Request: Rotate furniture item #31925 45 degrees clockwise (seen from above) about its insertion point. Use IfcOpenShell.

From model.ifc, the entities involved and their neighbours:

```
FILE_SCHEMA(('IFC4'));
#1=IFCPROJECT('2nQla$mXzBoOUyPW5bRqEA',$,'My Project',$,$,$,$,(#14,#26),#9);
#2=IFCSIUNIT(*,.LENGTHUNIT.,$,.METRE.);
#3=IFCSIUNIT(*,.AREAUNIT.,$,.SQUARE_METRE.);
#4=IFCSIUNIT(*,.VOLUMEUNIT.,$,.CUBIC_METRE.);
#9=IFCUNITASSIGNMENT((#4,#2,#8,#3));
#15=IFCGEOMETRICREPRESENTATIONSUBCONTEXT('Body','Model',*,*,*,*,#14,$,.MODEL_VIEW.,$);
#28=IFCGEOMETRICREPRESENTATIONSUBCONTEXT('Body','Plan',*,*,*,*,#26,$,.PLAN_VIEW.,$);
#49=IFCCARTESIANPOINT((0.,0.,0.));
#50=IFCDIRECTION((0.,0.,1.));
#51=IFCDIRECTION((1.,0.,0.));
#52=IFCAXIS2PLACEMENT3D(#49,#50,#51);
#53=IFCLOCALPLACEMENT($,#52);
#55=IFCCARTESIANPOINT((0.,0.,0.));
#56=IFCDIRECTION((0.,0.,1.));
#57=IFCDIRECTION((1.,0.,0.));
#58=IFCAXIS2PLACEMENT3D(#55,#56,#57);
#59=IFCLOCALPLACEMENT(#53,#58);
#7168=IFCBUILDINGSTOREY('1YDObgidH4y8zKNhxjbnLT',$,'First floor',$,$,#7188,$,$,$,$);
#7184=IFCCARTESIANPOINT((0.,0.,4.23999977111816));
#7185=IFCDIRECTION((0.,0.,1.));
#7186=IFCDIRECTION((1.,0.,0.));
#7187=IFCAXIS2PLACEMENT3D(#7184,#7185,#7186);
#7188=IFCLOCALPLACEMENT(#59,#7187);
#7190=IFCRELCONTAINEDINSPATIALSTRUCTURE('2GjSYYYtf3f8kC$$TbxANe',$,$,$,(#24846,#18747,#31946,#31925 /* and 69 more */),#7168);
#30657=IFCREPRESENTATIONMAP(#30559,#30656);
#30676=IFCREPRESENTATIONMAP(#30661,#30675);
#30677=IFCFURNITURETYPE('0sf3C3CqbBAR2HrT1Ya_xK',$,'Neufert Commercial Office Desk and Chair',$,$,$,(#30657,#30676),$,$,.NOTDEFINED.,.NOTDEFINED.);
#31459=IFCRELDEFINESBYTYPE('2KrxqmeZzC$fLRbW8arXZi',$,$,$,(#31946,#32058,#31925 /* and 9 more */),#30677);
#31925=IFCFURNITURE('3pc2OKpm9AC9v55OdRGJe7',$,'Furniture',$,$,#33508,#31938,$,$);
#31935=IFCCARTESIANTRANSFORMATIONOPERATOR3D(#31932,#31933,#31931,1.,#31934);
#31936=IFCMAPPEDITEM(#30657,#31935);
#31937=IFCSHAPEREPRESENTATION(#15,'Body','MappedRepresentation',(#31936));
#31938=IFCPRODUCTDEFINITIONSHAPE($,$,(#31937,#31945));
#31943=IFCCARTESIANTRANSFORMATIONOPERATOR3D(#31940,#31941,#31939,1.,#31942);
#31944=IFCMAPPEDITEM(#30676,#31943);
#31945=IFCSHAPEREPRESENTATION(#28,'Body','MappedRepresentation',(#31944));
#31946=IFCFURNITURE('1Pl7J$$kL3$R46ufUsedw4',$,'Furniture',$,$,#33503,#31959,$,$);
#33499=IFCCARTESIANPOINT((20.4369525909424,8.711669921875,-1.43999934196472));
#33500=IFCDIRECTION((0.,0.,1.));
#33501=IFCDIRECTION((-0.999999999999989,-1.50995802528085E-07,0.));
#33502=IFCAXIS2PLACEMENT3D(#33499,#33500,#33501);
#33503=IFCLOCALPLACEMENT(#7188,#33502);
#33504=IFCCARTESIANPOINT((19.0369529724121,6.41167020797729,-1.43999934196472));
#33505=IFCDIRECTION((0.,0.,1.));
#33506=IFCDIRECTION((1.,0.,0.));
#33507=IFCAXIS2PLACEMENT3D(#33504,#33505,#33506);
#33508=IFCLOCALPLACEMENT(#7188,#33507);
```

```python
import ifcopenshell
import ifcopenshell.api.geometry
import ifcopenshell.util.placement

model = ifcopenshell.open("model.ifc")

item = model.by_guid("3pc2OKpm9AC9v55OdRGJe7")
matrix = ifcopenshell.util.placement.get_local_placement(item.ObjectPlacement)
matrix = matrix @ ifcopenshell.util.placement.rotation(-45, "Z")
ifcopenshell.api.geometry.edit_object_placement(model, product=item, matrix=matrix, is_si=False)

print(ifcopenshell.util.placement.get_local_placement(item.ObjectPlacement).round(3) + 0.0)

model.write("model_v2.ifc")
```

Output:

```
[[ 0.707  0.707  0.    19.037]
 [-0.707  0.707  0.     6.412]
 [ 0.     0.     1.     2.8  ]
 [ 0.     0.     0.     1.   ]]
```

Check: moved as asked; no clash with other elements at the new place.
